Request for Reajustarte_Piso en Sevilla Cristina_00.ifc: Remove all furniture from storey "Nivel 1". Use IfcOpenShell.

First a look at what the model holds.

```python
import ifcopenshell
import ifcopenshell.util.element

model = ifcopenshell.open("Reajustarte_Piso en Sevilla Cristina_00.ifc")
print(model.schema)
storey = next(s for s in model.by_type("IfcBuildingStorey") if s.Name == "Nivel 1")
furniture = [e for e in ifcopenshell.util.element.get_decomposition(storey) if e.is_a("IfcFurnishingElement")]
seen = {}
for e in furniture:
    element_type = ifcopenshell.util.element.get_type(e)
    name = element_type.Name if element_type not in (None, e) else None
    seen[name] = seen.get(name, 0) + 1
for name, count in sorted(seen.items(), key=str):
    print(count, "x", name)
```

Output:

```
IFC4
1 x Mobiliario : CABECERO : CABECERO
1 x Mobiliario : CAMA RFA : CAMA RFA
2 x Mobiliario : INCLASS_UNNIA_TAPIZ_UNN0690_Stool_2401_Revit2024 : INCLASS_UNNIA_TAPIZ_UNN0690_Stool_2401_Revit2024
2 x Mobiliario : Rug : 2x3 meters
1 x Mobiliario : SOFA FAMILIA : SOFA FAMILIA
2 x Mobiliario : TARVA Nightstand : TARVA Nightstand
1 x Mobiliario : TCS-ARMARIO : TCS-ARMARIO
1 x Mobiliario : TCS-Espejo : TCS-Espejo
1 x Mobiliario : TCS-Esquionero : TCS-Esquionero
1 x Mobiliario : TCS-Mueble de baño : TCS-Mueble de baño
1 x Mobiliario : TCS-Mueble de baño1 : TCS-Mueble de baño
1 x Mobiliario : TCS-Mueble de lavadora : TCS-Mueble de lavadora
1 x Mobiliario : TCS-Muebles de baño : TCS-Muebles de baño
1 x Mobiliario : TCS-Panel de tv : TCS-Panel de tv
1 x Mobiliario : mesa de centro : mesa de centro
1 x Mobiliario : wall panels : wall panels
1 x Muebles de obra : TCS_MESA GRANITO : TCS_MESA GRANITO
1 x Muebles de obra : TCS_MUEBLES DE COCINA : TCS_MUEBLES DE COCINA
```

```python
import ifcopenshell
import ifcopenshell.api.root
import ifcopenshell.util.element

model = ifcopenshell.open("Reajustarte_Piso en Sevilla Cristina_00.ifc")

storey = next(s for s in model.by_type("IfcBuildingStorey") if s.Name == "Nivel 1")
furniture = [e for e in ifcopenshell.util.element.get_decomposition(storey) if e.is_a("IfcFurnishingElement")]

for e in furniture:
    ifcopenshell.api.root.remove_product(model, product=e)
print(len(furniture), "removed")

model.write("Reajustarte_Piso en Sevilla Cristina_00-out.ifc")
```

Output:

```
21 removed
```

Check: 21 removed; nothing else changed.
